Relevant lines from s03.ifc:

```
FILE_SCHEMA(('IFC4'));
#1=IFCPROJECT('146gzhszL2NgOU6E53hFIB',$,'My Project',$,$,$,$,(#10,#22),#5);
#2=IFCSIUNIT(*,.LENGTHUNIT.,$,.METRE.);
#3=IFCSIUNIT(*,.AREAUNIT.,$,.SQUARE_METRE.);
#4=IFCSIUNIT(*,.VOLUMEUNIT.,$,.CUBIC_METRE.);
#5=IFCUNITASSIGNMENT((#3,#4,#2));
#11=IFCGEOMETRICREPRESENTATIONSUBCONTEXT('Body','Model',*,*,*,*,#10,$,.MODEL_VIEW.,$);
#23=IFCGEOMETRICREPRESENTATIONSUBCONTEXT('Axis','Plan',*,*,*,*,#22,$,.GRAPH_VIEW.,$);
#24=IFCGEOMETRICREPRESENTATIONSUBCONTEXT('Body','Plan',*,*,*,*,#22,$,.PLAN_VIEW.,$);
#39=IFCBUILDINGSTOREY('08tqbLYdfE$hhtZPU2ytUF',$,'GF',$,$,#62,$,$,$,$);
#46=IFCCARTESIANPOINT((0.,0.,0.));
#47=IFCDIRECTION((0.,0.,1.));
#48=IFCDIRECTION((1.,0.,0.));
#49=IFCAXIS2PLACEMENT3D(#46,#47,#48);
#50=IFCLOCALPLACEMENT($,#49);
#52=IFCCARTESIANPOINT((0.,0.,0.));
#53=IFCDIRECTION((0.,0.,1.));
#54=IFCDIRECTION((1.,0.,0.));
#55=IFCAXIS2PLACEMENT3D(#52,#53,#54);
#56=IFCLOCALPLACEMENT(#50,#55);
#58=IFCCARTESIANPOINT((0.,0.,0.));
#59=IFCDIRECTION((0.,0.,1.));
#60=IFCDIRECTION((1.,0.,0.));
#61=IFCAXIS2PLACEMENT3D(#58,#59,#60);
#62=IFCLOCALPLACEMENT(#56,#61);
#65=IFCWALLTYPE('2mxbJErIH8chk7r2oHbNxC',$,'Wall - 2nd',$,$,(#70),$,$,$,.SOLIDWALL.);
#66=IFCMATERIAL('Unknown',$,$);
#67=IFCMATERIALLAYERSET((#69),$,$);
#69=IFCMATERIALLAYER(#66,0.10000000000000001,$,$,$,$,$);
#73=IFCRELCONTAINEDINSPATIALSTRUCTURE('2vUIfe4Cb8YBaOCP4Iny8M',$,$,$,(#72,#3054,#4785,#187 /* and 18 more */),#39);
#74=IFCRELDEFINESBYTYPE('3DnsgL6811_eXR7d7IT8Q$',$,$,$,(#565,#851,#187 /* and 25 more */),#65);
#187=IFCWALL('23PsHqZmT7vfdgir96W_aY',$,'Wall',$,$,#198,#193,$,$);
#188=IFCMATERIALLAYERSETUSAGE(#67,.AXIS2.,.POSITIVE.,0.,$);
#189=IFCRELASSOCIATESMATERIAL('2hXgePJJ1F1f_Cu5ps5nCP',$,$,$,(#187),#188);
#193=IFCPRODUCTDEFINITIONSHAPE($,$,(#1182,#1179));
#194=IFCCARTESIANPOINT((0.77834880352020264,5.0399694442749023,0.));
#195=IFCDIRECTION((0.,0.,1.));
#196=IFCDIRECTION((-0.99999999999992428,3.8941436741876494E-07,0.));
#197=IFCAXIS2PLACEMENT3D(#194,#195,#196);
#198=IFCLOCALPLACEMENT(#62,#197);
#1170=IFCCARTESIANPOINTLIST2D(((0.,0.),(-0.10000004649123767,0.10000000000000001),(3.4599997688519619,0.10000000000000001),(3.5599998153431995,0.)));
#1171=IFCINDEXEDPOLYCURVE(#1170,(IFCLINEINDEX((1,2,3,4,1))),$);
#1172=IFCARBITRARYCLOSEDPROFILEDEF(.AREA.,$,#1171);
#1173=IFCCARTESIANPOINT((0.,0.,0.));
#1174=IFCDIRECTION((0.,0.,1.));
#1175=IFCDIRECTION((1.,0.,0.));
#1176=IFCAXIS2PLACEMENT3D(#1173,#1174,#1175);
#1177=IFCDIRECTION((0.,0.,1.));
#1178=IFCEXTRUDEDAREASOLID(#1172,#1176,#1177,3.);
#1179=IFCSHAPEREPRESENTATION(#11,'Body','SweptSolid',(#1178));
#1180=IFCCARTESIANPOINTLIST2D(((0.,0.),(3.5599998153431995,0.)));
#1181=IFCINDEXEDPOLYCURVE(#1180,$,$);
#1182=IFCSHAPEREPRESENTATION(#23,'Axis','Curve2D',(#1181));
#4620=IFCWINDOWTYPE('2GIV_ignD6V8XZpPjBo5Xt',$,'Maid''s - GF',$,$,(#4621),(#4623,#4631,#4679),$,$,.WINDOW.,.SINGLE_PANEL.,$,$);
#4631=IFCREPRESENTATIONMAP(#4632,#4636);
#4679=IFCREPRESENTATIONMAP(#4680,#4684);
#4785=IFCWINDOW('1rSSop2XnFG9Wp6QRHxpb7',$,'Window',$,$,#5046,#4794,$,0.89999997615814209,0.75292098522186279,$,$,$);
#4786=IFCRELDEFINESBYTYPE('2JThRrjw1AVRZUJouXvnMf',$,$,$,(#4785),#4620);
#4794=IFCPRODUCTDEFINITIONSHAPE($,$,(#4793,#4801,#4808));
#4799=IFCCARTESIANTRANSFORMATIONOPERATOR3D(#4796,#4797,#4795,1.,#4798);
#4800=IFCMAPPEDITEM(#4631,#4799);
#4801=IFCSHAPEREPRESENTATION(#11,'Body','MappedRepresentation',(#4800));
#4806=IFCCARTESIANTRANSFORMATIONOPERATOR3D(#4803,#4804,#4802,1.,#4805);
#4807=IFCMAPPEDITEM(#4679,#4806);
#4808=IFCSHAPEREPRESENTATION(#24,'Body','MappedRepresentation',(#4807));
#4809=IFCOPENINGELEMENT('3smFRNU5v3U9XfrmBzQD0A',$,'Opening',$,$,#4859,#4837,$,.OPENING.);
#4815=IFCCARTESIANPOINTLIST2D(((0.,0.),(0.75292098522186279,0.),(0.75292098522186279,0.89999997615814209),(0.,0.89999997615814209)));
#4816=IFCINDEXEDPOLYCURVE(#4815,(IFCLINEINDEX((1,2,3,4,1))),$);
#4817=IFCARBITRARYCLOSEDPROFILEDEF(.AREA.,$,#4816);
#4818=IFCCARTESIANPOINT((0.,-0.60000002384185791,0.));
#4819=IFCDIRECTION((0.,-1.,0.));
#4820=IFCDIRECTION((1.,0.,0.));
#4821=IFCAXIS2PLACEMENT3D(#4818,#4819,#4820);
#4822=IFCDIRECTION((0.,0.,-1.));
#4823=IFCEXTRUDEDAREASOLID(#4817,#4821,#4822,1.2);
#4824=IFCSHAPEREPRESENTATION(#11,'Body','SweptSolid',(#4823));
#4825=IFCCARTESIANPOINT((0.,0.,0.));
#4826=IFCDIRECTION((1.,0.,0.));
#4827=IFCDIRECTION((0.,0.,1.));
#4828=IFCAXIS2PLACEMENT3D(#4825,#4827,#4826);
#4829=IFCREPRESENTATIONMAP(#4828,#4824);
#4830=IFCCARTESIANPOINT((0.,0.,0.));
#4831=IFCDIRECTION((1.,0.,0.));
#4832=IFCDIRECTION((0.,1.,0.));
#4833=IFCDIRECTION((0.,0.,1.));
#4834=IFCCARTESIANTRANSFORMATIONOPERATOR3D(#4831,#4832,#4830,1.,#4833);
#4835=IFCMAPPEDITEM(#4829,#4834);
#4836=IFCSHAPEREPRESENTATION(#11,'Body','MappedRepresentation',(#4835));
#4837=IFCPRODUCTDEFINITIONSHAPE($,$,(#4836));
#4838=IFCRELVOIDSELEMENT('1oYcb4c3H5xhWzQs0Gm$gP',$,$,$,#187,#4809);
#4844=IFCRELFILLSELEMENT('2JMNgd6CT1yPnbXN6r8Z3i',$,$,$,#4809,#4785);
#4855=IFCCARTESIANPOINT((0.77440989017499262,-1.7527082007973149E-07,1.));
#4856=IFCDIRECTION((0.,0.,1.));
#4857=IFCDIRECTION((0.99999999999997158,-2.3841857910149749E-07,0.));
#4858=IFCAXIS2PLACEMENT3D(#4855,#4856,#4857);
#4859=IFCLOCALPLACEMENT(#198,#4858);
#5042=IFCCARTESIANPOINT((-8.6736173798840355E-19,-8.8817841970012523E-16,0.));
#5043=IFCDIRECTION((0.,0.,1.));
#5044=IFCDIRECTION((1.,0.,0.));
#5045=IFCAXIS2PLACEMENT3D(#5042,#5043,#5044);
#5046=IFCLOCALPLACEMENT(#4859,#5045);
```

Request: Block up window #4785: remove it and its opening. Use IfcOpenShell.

```python
import ifcopenshell
import ifcopenshell.api.feature
import ifcopenshell.api.root
import ifcopenshell.geom
import ifcopenshell.util.shape

model = ifcopenshell.open("s03.ifc")
settings = ifcopenshell.geom.settings()


def volume(element):
    """Net volume in cubic metres, openings subtracted."""
    shape = ifcopenshell.geom.create_shape(settings, element)
    return ifcopenshell.util.shape.get_volume(shape.geometry)


window = model.by_guid("1rSSop2XnFG9Wp6QRHxpb7")
opening = window.FillsVoids[0].RelatingOpeningElement
wall = opening.VoidsElements[0].RelatingBuildingElement
before = volume(wall)

ifcopenshell.api.root.remove_product(model, product=window)
ifcopenshell.api.feature.remove_feature(model, feature=opening)

after = volume(wall)

print(f"wall volume {before:.3f} -> {after:.3f} m3")

model.write("s03_updated.ifc")
```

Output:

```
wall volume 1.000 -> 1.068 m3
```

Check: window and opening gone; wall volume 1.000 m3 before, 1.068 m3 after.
